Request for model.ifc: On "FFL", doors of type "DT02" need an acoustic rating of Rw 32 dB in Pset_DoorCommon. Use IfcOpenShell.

First a look at what the model holds.

```python
import ifcopenshell
import ifcopenshell.util.element

model = ifcopenshell.open("model.ifc")
print(model.schema)
storey = next(s for s in model.by_type("IfcBuildingStorey") if s.Name == "FFL")
doors = [e for e in ifcopenshell.util.element.get_decomposition(storey) if e.is_a("IfcDoor")]
seen = {}
for e in doors:
    element_type = ifcopenshell.util.element.get_type(e)
    key = (element_type.Name if element_type != e and element_type else None, ifcopenshell.util.element.get_pset(e, "Pset_DoorCommon", "AcousticRating"))
    seen[key] = seen.get(key, 0) + 1
for (name, value), count in sorted(seen.items(), key=str):
    print(count, "x", name, "|", value)
```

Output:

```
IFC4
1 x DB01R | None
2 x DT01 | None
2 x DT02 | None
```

```python
import ifcopenshell
import ifcopenshell.api.pset
import ifcopenshell.util.element

model = ifcopenshell.open("model.ifc")

storey = next(s for s in model.by_type("IfcBuildingStorey") if s.Name == "FFL")
doors = [e for e in ifcopenshell.util.element.get_decomposition(storey) if e.is_a("IfcDoor")]

count = 0
for e in doors:
    element_type = ifcopenshell.util.element.get_type(e)
    if element_type in (None, e) or element_type.Name != "DT02":
        continue
    # add_pset returns the element's existing set when there is one.
    pset = ifcopenshell.api.pset.add_pset(model, product=e, name="Pset_DoorCommon")
    ifcopenshell.api.pset.edit_pset(model, pset=pset, properties={"AcousticRating": "Rw 32 dB"})
    count += 1

print(count, "doors updated")

model.write("model_updated.ifc")
```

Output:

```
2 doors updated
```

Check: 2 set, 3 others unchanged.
